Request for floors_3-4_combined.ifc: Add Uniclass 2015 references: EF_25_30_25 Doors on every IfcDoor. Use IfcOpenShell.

First a look at what the model holds.

```python
import ifcopenshell

model = ifcopenshell.open("floors_3-4_combined.ifc")
print(model.schema)
print("classifications:", [c.Name for c in model.by_type("IfcClassification")])
for ifc_class in ("IfcDoor", "IfcRoof", "IfcStair", "IfcWall", "IfcWindow"):
    print(ifc_class, len(model.by_type(ifc_class)))
```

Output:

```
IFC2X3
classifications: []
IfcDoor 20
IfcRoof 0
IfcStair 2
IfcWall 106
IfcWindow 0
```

```python
import ifcopenshell
import ifcopenshell.api.classification

model = ifcopenshell.open("floors_3-4_combined.ifc")

# IFC2X3 requires Source and Edition and has no link from the project to the system.
system = model.create_entity("IfcClassification", Source="NBS", Edition="2015", Name="Uniclass 2015")

codes = {
    "IfcDoor": ("EF_25_30_25", "Doors"),
}
for ifc_class, (code, name) in codes.items():
    products = model.by_type(ifc_class)
    ifcopenshell.api.classification.add_reference(
        model, products=products, classification=system, identification=code, name=name
    )
    print(code, len(products))

model.write("floors_3-4_combined_edited.ifc")
```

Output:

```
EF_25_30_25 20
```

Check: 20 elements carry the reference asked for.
